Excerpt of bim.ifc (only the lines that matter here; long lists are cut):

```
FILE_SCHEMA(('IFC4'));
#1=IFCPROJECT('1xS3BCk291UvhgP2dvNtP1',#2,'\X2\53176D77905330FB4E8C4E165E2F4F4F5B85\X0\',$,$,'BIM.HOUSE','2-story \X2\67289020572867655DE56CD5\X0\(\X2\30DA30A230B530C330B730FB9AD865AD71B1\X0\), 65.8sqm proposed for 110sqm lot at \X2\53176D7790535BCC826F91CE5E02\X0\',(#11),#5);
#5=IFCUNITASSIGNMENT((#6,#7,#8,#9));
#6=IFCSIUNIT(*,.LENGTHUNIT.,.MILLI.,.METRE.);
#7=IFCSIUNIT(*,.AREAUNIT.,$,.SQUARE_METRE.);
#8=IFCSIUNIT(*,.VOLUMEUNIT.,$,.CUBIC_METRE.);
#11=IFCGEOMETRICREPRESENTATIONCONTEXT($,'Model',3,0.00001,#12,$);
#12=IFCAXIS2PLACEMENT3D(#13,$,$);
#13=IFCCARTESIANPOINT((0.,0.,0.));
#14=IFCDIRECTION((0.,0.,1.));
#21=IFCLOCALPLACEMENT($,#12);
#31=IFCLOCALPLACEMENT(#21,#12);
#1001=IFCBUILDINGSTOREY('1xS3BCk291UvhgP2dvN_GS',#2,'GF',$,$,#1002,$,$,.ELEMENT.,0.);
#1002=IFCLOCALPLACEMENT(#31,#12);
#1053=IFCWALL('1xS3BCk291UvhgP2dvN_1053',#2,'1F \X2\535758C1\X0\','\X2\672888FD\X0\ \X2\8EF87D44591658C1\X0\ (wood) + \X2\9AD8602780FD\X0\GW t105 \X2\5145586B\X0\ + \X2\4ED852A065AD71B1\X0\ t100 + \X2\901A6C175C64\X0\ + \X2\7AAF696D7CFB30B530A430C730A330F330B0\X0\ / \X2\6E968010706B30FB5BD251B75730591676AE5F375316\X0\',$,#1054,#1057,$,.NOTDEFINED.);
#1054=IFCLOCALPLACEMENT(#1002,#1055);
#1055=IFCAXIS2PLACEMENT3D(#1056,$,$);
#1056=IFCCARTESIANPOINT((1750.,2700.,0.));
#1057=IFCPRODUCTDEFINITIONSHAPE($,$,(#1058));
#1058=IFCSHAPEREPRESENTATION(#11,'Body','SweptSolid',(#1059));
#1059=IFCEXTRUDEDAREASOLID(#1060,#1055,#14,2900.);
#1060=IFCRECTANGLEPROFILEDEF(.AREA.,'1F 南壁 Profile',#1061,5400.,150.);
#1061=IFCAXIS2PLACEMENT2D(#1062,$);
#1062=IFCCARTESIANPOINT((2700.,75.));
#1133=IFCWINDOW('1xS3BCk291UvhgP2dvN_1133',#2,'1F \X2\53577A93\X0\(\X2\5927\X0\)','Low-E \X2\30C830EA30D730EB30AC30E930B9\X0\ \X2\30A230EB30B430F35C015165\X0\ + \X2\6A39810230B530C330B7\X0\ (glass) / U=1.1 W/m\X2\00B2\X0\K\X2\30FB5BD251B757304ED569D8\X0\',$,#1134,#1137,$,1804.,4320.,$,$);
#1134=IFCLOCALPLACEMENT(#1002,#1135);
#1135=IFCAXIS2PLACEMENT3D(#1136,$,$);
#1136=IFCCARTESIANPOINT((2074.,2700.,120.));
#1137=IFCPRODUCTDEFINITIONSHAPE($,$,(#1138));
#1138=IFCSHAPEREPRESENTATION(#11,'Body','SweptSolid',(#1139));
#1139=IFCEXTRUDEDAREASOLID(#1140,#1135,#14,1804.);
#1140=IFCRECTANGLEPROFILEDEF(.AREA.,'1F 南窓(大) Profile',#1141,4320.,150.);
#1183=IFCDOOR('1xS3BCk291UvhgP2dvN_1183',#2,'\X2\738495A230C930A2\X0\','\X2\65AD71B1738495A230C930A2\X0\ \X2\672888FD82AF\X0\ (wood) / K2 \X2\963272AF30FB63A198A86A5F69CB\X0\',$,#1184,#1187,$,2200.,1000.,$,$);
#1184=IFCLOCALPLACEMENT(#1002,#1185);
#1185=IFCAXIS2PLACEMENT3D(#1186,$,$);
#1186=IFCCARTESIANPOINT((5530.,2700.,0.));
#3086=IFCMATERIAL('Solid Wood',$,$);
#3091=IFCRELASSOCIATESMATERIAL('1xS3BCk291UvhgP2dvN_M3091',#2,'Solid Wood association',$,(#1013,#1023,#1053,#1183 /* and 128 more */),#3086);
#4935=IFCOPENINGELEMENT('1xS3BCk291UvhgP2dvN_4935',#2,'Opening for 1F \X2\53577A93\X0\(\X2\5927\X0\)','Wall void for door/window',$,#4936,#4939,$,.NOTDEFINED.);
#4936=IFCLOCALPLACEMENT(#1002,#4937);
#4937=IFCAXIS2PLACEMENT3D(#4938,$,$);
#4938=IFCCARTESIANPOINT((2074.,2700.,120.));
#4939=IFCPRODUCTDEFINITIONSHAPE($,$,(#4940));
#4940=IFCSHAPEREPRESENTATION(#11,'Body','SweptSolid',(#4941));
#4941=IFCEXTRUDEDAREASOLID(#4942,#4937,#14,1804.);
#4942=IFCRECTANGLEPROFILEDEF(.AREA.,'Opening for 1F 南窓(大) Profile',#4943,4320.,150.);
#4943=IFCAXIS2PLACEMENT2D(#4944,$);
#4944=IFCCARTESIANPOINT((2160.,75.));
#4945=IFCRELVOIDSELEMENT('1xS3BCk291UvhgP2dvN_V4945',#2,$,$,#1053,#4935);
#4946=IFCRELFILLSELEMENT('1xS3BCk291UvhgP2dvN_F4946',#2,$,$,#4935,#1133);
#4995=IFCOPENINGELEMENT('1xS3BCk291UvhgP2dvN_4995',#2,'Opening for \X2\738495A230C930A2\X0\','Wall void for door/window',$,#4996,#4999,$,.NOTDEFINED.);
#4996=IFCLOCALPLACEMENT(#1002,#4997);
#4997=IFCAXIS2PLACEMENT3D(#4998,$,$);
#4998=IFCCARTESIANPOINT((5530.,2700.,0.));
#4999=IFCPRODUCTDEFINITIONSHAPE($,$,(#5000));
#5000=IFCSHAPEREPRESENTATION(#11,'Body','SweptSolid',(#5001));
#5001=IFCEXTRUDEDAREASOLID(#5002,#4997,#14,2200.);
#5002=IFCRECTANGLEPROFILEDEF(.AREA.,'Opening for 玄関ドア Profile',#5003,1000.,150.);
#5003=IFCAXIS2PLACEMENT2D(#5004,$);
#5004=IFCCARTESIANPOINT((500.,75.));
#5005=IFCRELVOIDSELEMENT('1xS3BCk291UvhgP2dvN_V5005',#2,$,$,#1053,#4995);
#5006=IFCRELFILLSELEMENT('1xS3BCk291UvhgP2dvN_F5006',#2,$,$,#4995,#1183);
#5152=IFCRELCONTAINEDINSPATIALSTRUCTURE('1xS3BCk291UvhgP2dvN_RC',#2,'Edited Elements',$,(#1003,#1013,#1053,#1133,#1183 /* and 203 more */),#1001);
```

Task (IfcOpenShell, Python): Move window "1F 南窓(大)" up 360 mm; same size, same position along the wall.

```python
import numpy as np
import ifcopenshell
import ifcopenshell.api.geometry
import ifcopenshell.util.placement
import ifcopenshell.util.unit

model = ifcopenshell.open("bim.ifc")
unit_scale = ifcopenshell.util.unit.calculate_unit_scale(model)

window = model.by_guid("1xS3BCk291UvhgP2dvN_1133")
opening = window.FillsVoids[0].RelatingOpeningElement
dz = 360.0

shift = np.array([0.0, 0.0, dz])
# The window is not placed relative to its opening, so move both.
for product in (opening, window):
    matrix = ifcopenshell.util.placement.get_local_placement(product.ObjectPlacement)
    matrix[:3, 3] += shift
    ifcopenshell.api.geometry.edit_object_placement(model, product=product, matrix=matrix, is_si=False)

print(f"moved by {dz * unit_scale:+.3f} m")

model.write("bim_v2.ifc")
```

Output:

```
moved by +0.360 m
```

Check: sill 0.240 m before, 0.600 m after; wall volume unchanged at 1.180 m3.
